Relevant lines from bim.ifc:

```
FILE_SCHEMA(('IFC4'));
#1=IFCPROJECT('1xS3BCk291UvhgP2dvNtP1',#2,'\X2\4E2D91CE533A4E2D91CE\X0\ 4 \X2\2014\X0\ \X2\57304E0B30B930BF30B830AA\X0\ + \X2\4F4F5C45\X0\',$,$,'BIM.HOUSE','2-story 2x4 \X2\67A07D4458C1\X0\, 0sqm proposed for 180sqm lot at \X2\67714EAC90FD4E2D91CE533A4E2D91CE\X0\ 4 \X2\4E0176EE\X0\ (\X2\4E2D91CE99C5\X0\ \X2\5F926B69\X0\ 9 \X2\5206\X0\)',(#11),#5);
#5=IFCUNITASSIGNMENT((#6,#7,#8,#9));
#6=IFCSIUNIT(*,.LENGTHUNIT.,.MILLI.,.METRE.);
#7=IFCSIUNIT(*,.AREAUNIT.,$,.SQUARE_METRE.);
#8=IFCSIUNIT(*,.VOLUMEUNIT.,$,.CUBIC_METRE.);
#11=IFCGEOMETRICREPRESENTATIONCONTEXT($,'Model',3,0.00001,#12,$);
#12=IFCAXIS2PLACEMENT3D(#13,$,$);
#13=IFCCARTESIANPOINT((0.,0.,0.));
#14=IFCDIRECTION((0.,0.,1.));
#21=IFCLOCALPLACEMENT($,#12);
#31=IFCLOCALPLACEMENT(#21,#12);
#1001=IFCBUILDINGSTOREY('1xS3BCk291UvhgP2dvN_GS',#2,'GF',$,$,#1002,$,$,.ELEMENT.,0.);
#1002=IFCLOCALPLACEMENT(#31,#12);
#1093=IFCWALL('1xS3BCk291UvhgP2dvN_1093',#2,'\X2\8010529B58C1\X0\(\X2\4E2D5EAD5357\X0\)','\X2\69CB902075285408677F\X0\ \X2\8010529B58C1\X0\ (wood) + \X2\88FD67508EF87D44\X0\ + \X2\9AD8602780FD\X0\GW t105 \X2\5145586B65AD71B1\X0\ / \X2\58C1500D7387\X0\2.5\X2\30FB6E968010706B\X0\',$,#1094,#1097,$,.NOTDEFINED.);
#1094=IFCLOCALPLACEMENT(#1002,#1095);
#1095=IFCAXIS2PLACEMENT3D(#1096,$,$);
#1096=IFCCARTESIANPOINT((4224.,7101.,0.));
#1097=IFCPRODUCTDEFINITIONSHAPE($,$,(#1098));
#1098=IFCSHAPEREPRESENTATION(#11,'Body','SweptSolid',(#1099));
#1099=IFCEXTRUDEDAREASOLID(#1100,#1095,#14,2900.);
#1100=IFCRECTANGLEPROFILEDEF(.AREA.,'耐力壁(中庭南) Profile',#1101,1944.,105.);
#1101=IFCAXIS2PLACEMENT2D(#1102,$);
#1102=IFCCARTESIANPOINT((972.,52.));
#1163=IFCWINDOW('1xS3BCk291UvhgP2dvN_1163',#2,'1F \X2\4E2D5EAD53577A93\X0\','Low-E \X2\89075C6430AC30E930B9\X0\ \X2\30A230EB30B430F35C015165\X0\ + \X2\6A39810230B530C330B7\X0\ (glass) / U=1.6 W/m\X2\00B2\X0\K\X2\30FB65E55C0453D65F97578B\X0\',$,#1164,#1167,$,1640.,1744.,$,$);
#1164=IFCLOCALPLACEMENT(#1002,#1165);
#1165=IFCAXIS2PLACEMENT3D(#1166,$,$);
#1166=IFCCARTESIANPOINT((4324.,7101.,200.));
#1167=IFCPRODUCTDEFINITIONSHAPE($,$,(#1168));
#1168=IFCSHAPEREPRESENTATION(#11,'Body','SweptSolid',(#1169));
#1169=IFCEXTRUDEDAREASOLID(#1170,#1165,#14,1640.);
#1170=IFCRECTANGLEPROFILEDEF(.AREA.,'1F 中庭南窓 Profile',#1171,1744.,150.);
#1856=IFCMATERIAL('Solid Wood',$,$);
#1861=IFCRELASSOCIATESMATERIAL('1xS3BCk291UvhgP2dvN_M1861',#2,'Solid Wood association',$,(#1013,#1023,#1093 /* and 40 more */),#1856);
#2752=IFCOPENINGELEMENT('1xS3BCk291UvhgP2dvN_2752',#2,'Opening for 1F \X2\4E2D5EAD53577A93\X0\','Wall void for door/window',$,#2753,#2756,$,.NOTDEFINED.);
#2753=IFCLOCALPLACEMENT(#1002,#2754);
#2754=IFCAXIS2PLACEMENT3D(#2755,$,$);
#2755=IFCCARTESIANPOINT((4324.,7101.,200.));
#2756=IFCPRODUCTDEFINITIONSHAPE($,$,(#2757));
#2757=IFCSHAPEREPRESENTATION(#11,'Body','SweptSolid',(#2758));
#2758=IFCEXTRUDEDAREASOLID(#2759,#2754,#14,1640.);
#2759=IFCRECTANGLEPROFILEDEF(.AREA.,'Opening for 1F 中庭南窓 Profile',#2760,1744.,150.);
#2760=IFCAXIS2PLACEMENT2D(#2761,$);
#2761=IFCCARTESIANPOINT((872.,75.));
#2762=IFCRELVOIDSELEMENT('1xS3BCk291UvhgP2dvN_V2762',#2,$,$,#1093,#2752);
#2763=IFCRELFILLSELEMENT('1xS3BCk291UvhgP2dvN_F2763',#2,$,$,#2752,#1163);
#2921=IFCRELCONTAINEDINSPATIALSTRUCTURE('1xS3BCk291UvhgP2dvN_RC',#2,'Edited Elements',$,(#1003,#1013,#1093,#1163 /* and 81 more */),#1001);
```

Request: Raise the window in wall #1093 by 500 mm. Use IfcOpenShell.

```python
import numpy as np
import ifcopenshell
import ifcopenshell.api.geometry
import ifcopenshell.util.placement
import ifcopenshell.util.unit

model = ifcopenshell.open("bim.ifc")
unit_scale = ifcopenshell.util.unit.calculate_unit_scale(model)

window = model.by_id(1163)
opening = window.FillsVoids[0].RelatingOpeningElement
dz = 0.5 / unit_scale

shift = np.array([0.0, 0.0, dz])
# The window is not placed relative to its opening, so move both.
for product in (opening, window):
    matrix = ifcopenshell.util.placement.get_local_placement(product.ObjectPlacement)
    matrix[:3, 3] += shift
    ifcopenshell.api.geometry.edit_object_placement(model, product=product, matrix=matrix, is_si=False)

print(f"moved by {dz * unit_scale:+.3f} m")

model.write("bim_edited.ifc")
```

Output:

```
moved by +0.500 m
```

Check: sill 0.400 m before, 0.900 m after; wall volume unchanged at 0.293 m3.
